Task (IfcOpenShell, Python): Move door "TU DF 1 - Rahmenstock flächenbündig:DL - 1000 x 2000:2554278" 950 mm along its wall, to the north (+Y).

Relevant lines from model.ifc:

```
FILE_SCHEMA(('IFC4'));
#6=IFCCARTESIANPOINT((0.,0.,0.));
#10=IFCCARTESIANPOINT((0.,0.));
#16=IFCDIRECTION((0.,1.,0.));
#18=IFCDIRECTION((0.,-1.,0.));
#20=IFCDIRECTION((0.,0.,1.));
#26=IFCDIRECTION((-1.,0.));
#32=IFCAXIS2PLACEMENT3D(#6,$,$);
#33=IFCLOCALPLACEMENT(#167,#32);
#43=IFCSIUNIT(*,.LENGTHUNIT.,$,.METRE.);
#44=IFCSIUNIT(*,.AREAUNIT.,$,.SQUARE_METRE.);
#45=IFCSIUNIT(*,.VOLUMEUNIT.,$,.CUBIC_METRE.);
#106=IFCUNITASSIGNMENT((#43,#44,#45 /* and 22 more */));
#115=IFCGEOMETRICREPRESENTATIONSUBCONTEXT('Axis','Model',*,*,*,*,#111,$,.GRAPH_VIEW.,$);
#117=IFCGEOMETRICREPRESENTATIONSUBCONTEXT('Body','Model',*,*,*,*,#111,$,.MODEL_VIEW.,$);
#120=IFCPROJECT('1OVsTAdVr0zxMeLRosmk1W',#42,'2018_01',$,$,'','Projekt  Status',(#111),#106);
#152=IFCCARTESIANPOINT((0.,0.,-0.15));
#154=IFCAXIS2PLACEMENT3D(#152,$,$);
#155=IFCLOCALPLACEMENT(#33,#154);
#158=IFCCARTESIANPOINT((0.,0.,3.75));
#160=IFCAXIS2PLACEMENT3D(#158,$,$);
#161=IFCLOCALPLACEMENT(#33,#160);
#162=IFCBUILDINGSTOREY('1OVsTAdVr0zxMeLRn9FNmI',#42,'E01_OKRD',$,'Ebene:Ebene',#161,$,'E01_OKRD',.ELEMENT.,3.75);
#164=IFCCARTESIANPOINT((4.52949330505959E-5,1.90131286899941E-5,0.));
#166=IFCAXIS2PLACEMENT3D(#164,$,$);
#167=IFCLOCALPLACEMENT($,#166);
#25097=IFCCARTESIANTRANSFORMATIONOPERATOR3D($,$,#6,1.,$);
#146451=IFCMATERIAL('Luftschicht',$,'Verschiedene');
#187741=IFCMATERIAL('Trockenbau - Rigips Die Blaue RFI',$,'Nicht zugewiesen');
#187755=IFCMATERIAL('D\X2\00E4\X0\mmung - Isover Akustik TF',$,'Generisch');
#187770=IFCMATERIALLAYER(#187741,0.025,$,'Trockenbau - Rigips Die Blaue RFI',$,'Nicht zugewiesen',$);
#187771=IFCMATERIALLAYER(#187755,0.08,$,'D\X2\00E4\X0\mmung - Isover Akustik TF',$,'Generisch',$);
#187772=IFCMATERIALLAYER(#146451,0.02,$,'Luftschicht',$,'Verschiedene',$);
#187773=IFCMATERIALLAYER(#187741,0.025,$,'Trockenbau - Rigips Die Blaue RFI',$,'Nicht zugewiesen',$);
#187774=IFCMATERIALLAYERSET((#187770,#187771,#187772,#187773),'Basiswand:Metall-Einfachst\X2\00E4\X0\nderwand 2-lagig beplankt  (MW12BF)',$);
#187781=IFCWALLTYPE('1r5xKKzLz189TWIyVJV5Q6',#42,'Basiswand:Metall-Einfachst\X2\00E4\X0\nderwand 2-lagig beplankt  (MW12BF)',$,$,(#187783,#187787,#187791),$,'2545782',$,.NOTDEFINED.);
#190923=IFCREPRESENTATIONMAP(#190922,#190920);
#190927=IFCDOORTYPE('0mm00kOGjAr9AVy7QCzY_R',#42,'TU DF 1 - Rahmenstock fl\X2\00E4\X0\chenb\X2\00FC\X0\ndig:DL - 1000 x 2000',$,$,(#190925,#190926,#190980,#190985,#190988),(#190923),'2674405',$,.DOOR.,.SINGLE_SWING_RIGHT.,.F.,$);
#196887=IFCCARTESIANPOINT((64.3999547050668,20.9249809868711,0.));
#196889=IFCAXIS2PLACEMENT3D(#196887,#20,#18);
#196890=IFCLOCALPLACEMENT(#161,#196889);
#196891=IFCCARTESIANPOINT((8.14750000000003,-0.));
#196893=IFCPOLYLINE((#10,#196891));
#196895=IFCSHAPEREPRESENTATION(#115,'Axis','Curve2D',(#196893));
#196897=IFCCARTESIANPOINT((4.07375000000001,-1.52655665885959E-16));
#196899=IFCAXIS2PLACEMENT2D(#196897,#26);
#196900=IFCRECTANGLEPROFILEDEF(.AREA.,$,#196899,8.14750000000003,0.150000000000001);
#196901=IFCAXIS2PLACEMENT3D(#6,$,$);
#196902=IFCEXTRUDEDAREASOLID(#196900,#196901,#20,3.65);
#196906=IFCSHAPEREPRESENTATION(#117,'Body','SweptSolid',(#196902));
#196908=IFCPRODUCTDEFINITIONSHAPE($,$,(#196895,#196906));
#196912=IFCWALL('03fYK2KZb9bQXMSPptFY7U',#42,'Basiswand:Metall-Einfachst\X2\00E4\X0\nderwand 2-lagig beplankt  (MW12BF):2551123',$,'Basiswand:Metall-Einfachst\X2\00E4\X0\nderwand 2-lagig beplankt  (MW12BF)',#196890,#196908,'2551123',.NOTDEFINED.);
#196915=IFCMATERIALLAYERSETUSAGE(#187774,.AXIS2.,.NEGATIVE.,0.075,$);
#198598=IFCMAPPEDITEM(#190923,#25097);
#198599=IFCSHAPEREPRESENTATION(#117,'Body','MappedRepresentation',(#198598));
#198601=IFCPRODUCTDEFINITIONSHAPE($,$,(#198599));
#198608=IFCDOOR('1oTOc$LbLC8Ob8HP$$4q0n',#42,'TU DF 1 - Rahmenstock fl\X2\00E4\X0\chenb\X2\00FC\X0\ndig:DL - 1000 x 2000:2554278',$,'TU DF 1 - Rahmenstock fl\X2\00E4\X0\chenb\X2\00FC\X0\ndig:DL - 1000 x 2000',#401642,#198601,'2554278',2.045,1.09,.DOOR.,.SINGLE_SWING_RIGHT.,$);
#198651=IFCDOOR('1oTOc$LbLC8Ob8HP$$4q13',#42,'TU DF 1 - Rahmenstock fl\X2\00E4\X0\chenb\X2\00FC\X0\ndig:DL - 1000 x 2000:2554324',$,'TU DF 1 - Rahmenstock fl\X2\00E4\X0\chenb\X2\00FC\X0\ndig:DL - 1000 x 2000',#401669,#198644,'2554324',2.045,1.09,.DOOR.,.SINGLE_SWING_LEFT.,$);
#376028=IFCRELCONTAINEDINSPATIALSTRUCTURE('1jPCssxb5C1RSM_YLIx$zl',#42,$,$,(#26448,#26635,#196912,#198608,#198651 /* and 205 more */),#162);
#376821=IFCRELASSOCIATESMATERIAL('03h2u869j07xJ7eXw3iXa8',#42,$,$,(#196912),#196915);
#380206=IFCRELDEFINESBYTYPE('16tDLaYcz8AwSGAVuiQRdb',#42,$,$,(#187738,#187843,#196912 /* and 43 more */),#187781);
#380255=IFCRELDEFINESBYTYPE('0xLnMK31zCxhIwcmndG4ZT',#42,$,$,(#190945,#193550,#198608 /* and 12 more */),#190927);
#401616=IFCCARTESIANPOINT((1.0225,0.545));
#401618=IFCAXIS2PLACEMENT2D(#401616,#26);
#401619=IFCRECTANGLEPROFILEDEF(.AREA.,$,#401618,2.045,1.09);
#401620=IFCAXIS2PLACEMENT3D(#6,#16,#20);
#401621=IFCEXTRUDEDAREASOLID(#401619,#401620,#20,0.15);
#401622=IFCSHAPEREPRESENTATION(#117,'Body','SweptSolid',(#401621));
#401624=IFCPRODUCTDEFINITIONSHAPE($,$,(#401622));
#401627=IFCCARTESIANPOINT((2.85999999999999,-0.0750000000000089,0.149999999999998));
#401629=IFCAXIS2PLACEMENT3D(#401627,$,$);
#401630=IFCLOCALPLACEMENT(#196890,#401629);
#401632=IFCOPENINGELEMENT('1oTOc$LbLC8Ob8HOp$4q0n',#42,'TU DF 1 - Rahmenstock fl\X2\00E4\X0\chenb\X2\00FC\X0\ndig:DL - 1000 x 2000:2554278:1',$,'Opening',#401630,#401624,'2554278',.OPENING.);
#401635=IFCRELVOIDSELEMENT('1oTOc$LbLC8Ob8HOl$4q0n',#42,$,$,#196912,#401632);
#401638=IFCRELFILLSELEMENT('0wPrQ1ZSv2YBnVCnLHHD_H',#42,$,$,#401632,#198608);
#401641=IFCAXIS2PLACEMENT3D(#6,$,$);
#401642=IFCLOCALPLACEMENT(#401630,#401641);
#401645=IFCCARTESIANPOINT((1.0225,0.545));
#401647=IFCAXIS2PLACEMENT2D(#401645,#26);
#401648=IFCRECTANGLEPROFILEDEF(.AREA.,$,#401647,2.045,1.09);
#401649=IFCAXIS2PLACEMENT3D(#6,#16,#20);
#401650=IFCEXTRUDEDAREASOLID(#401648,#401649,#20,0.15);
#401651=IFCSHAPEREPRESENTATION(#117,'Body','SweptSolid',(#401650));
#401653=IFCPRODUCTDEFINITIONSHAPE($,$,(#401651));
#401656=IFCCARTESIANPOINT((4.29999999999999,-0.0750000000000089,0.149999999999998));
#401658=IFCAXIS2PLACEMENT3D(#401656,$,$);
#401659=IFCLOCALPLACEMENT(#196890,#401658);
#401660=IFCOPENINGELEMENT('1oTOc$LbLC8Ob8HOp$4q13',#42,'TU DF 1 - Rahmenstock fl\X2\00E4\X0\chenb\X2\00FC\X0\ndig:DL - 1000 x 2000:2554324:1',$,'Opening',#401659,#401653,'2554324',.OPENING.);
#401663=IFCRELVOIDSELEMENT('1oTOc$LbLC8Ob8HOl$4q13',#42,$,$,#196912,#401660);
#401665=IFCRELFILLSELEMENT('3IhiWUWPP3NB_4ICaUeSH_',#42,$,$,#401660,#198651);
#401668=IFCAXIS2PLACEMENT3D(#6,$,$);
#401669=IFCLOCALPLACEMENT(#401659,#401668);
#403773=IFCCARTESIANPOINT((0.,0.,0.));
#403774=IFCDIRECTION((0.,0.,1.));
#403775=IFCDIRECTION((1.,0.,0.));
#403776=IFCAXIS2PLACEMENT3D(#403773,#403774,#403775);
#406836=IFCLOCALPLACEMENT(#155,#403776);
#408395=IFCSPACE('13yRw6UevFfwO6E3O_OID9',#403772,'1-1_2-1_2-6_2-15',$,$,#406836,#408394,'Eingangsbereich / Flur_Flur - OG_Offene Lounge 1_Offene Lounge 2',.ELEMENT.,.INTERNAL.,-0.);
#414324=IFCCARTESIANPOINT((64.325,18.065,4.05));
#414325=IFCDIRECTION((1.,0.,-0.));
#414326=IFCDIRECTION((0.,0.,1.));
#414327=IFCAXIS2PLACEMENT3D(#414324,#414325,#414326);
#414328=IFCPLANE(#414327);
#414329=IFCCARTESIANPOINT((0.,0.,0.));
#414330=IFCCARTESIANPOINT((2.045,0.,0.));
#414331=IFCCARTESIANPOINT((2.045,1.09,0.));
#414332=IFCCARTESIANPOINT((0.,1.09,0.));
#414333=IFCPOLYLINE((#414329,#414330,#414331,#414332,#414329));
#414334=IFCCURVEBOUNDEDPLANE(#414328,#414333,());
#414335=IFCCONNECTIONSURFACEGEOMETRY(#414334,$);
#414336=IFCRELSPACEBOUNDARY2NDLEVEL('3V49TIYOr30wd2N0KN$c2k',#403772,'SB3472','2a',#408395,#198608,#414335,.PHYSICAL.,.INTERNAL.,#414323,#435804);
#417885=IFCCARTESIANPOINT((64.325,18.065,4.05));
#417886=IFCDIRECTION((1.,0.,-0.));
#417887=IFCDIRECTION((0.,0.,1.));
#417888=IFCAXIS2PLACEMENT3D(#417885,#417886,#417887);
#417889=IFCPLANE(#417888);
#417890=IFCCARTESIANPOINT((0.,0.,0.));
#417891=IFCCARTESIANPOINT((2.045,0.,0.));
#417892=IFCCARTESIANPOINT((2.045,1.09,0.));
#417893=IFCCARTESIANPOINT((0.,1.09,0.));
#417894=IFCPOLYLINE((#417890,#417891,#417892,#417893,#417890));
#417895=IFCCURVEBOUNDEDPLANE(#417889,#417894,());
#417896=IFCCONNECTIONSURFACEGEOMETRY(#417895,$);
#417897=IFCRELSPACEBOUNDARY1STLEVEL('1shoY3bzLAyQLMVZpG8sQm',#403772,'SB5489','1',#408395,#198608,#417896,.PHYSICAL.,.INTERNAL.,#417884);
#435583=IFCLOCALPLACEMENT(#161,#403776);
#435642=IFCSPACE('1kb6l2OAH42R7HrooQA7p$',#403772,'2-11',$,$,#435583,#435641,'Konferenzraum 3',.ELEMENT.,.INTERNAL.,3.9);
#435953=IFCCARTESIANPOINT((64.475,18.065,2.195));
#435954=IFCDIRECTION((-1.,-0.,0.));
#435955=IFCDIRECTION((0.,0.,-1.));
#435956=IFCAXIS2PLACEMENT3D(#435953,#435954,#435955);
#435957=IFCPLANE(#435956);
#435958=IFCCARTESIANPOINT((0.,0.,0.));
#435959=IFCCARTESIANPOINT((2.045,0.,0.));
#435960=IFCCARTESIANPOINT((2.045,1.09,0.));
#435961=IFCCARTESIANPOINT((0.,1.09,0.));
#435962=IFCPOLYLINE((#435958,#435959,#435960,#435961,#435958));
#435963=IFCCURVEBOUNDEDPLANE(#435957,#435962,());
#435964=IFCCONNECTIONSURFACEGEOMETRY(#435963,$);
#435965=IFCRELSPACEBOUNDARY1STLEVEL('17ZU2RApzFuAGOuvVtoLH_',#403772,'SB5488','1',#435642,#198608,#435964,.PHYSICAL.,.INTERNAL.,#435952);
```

```python
import numpy as np
import ifcopenshell
import ifcopenshell.api.geometry
import ifcopenshell.util.placement

model = ifcopenshell.open("model.ifc")

door = model.by_guid("1oTOc$LbLC8Ob8HP$$4q0n")
opening = door.FillsVoids[0].RelatingOpeningElement
wall = opening.VoidsElements[0].RelatingBuildingElement

wall_matrix = ifcopenshell.util.placement.get_local_placement(wall.ObjectPlacement)
shift = wall_matrix[:3, 0] * -0.95
before = ifcopenshell.util.placement.get_local_placement(door.ObjectPlacement)[:3, 3].copy()

# The door is placed relative to its opening, so it follows when the opening moves.
matrix = ifcopenshell.util.placement.get_local_placement(opening.ObjectPlacement)
matrix[:3, 3] += shift
ifcopenshell.api.geometry.edit_object_placement(
    model, product=opening, matrix=matrix, is_si=False, should_transform_children=True
)

# Space boundary surfaces are stored in each space's coordinates; move them too.
for rel in door.ProvidesBoundaries:
    if not rel.ConnectionGeometry:
        continue
    surface = rel.ConnectionGeometry.SurfaceOnRelatingElement.BasisSurface
    space_matrix = ifcopenshell.util.placement.get_local_placement(rel.RelatingSpace.ObjectPlacement)
    point = np.array(surface.Position.Location.Coordinates) + space_matrix[:3, :3].T @ shift
    surface.Position = model.createIfcAxis2Placement3D(
        model.createIfcCartesianPoint(point.tolist()), surface.Position.Axis, surface.Position.RefDirection
    )

after = ifcopenshell.util.placement.get_local_placement(door.ObjectPlacement)[:3, 3]
print("door moved by", (after - before).round(3) + 0.0)

model.write("model_edited.ifc")
```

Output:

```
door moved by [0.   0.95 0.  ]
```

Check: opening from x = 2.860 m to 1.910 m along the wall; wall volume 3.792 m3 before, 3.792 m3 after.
